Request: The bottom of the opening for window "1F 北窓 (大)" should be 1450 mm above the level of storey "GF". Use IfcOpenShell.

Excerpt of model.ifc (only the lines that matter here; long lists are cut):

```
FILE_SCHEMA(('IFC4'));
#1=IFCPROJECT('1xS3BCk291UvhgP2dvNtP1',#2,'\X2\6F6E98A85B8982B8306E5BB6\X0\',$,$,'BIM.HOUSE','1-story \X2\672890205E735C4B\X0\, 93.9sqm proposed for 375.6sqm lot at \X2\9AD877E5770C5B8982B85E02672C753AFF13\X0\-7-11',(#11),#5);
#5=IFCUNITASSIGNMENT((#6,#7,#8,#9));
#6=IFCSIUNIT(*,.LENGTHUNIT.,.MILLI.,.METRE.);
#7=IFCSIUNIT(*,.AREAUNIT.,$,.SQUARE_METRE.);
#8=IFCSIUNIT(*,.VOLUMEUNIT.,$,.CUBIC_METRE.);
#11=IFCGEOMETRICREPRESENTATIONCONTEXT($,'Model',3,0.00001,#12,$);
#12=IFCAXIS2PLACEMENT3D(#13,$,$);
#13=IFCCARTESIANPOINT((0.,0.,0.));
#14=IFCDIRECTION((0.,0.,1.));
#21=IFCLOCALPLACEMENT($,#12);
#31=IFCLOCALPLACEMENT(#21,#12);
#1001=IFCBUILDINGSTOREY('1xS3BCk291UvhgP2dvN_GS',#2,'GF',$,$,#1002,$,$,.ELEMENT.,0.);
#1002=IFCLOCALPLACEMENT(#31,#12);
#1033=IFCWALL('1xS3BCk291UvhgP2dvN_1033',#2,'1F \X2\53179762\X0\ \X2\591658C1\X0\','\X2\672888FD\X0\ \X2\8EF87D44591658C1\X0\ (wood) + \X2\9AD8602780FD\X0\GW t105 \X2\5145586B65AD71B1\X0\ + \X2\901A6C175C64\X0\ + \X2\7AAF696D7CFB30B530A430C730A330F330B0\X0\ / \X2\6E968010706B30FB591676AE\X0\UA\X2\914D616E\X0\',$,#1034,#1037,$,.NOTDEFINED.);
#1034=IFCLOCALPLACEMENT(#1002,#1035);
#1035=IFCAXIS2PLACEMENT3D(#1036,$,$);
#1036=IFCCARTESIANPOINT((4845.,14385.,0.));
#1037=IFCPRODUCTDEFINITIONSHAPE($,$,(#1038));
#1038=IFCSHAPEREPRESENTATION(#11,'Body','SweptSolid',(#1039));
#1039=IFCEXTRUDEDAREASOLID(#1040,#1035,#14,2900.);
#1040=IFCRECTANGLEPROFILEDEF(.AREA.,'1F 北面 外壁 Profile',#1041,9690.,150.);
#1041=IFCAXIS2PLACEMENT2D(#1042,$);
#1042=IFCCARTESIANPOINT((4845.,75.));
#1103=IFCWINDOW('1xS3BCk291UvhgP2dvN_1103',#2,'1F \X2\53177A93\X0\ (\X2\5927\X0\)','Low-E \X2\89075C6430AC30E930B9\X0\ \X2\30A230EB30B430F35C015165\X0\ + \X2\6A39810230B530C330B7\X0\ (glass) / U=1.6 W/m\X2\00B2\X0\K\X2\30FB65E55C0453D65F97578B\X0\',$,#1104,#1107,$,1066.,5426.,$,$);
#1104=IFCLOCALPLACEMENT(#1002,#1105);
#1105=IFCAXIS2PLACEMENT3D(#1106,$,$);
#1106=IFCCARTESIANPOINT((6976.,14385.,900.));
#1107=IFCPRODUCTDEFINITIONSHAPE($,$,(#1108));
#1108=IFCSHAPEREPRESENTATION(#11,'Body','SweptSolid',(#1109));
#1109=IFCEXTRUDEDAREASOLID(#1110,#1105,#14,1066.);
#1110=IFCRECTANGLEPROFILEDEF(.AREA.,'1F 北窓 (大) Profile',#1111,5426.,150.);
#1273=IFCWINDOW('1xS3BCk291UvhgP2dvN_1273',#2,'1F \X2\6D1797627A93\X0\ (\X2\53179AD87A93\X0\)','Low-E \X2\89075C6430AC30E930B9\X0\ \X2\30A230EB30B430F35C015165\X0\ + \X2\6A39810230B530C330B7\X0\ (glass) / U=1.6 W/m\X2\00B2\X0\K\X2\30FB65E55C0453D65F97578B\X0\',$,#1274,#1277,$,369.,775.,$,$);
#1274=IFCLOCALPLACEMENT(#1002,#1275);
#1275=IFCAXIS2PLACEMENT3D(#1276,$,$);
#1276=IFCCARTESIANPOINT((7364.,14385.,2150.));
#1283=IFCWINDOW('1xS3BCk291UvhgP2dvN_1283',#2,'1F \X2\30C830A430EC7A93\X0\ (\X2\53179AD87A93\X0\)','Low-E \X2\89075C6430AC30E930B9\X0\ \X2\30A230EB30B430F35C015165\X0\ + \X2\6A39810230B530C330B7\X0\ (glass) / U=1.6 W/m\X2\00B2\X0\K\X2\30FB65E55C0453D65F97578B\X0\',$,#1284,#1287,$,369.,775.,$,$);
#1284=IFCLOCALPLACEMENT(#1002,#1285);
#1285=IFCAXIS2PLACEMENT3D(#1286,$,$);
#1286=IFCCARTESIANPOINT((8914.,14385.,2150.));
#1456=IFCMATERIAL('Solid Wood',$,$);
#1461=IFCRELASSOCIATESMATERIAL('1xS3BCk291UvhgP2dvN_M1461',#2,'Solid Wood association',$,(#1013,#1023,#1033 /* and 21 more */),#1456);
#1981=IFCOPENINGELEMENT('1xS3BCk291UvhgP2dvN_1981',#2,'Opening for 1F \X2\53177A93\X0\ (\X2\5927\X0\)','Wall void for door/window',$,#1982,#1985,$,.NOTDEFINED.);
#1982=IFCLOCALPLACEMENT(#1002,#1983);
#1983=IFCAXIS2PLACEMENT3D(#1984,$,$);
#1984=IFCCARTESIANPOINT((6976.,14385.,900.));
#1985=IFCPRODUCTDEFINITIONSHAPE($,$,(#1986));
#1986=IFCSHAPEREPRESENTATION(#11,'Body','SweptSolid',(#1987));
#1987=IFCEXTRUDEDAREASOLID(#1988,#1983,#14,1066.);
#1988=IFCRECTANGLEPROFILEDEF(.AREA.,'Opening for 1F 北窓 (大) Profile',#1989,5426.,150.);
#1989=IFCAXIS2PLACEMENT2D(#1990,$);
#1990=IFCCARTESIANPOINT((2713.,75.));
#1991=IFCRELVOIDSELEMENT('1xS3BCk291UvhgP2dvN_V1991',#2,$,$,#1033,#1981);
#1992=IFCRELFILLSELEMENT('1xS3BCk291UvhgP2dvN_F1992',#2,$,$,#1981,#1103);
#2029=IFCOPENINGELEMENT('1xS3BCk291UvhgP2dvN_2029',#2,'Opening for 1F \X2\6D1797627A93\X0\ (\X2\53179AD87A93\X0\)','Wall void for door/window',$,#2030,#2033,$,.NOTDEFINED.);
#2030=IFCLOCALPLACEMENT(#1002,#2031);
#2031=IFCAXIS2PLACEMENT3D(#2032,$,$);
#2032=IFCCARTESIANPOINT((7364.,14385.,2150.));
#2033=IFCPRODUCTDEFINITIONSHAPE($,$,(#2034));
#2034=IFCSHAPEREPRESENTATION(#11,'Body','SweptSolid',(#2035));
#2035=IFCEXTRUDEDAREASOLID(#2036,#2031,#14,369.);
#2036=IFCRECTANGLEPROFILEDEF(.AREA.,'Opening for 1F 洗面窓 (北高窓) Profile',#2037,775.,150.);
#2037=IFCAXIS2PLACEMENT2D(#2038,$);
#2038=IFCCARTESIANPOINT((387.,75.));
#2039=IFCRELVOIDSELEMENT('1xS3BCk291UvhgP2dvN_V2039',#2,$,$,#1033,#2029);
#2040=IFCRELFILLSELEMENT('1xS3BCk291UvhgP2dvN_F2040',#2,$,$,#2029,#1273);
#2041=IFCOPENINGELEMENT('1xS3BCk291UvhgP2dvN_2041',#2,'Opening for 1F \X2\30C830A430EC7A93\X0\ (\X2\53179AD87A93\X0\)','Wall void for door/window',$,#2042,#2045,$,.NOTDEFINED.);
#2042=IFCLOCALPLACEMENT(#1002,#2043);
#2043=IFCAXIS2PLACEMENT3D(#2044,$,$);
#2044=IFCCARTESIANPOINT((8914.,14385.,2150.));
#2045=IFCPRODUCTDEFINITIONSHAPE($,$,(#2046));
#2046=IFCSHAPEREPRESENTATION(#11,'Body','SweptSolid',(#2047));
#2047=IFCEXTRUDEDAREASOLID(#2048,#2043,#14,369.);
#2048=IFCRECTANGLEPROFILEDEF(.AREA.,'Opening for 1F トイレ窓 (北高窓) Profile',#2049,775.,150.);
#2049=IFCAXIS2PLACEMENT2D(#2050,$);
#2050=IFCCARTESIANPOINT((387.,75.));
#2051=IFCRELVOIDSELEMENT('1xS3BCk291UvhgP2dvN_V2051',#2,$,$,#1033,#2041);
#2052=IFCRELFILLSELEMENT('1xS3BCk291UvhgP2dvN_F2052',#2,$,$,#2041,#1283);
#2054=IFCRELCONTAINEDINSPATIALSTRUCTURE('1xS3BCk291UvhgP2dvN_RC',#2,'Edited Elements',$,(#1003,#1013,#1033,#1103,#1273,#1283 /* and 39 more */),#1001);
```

```python
import numpy as np
import ifcopenshell
import ifcopenshell.api.geometry
import ifcopenshell.geom
import ifcopenshell.util.element
import ifcopenshell.util.placement
import ifcopenshell.util.shape
import ifcopenshell.util.unit

model = ifcopenshell.open("model.ifc")
unit_scale = ifcopenshell.util.unit.calculate_unit_scale(model)

window = model.by_guid("1xS3BCk291UvhgP2dvN_1103")
opening = window.FillsVoids[0].RelatingOpeningElement
storey = ifcopenshell.util.element.get_container(window, ifc_class="IfcBuildingStorey")
level = ifcopenshell.util.placement.get_local_placement(storey.ObjectPlacement)[2, 3]

# The opening's origin need not be at the sill, so measure its lowest point.
shape = ifcopenshell.geom.create_shape(ifcopenshell.geom.settings(), opening)
bottom = ifcopenshell.util.shape.get_shape_bottom_elevation(shape, shape.geometry) / unit_scale
dz = level + 1.45 / unit_scale - bottom

shift = np.array([0.0, 0.0, dz])
# The window is not placed relative to its opening, so move both.
for product in (opening, window):
    matrix = ifcopenshell.util.placement.get_local_placement(product.ObjectPlacement)
    matrix[:3, 3] += shift
    ifcopenshell.api.geometry.edit_object_placement(model, product=product, matrix=matrix, is_si=False)

print(f"moved by {dz * unit_scale:+.3f} m")

model.write("model_updated.ifc")
```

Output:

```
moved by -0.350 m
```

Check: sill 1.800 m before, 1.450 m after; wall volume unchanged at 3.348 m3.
